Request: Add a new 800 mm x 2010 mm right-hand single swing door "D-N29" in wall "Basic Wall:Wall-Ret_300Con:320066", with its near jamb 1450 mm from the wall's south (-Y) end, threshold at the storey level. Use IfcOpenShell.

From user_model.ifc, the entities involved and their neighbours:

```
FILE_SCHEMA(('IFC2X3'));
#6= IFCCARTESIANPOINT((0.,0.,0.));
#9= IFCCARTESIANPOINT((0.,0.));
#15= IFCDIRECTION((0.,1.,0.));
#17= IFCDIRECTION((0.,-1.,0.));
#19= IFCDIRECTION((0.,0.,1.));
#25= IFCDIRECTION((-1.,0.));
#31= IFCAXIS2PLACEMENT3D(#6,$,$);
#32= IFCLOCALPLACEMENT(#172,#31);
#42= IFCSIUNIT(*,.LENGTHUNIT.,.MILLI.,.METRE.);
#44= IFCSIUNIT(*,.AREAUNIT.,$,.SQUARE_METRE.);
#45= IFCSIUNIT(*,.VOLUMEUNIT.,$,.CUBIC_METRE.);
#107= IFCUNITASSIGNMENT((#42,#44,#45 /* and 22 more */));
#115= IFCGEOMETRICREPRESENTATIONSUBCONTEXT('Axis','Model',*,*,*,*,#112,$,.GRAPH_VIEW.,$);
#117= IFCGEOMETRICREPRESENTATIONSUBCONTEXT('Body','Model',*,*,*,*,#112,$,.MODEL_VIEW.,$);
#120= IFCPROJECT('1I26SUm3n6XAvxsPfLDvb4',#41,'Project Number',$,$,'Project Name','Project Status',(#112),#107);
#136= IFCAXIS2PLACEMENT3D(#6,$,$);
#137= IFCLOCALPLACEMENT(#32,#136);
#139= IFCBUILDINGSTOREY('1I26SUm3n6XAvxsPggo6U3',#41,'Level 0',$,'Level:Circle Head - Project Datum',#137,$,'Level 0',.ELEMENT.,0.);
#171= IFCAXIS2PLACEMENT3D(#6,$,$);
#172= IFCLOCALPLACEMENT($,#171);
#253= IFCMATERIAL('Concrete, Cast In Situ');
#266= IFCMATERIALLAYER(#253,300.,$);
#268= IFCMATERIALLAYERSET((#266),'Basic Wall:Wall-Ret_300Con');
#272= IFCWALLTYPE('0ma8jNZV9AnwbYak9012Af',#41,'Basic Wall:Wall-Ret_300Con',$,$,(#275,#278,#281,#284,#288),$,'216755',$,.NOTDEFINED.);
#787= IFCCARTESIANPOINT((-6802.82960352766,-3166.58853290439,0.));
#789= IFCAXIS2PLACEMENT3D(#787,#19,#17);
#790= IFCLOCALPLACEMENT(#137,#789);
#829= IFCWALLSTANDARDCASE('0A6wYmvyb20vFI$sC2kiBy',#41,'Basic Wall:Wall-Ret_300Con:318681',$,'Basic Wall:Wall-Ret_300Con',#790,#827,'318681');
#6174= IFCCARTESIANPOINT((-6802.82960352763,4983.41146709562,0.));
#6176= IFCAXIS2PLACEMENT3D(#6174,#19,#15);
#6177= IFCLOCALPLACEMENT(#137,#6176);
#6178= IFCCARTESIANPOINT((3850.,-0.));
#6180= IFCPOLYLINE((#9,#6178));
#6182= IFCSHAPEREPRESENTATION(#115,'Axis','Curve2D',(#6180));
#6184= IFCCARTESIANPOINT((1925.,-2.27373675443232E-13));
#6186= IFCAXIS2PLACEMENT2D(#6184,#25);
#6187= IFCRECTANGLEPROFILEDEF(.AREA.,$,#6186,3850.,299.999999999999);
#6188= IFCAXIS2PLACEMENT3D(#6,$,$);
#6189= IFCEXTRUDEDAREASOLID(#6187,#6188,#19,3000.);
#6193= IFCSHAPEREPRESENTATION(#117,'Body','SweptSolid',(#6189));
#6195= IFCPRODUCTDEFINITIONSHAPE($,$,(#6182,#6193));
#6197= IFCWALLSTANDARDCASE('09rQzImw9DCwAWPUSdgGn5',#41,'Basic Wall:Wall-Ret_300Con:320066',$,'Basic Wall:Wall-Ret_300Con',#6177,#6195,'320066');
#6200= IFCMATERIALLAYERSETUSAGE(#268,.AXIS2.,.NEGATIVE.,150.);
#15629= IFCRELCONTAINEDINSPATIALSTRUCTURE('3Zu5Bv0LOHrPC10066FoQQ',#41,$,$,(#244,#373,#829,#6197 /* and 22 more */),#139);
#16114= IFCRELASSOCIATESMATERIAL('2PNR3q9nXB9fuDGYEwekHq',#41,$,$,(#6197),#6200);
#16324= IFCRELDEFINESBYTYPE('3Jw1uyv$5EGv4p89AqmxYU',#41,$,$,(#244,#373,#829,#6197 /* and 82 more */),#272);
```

```python
import numpy as np
import ifcopenshell
import ifcopenshell.api.feature
import ifcopenshell.api.geometry
import ifcopenshell.api.root
import ifcopenshell.api.spatial
import ifcopenshell.api.type
import ifcopenshell.geom
import ifcopenshell.util.element
import ifcopenshell.util.placement
import ifcopenshell.util.representation
import ifcopenshell.util.shape
import ifcopenshell.util.unit

model = ifcopenshell.open("user_model.ifc")
unit_scale = ifcopenshell.util.unit.calculate_unit_scale(model)
settings = ifcopenshell.geom.settings()


def volume(element):
    """Net volume in cubic metres, openings subtracted."""
    shape = ifcopenshell.geom.create_shape(settings, element)
    return ifcopenshell.util.shape.get_volume(shape.geometry)


wall = model.by_id(6197)
storey = ifcopenshell.util.element.get_container(wall, ifc_class="IfcBuildingStorey")
context = ifcopenshell.util.representation.get_context(model, "Model", "Body", "MODEL_VIEW")
before = volume(wall)

width, height, from_end, sill = 0.8, 2.01, 1.45, 0.0  # metres

# The wall runs along its own X axis, and the end named is its -X end.
wall_shape = ifcopenshell.geom.create_shape(settings, wall)
x, y, z = ifcopenshell.util.shape.get_vertices(wall_shape.geometry).T
start = x.min() + from_end
face, thickness = float(y.min()), float(y.max() - y.min())
wall_matrix = ifcopenshell.util.placement.get_local_placement(wall.ObjectPlacement)
level = ifcopenshell.util.placement.get_local_placement(storey.ObjectPlacement)[2, 3]


def in_wall(x, y):
    """Placement at x, y metres in the wall's axes, at sill height."""
    matrix = wall_matrix.copy()
    matrix[:, 3] = wall_matrix @ np.array([x / unit_scale, y / unit_scale, 0.0, 1.0])
    matrix[2, 3] = level + sill / unit_scale
    return matrix


# Opening: a box that overshoots both wall faces by 50 mm.
opening = ifcopenshell.api.root.create_entity(model, ifc_class="IfcOpeningElement")
box = ifcopenshell.api.geometry.add_wall_representation(
    model, context=context, length=width, height=height, thickness=thickness + 0.1
)
ifcopenshell.api.geometry.assign_representation(model, product=opening, representation=box)
ifcopenshell.api.geometry.edit_object_placement(model, product=opening, matrix=in_wall(start, face - 0.05), is_si=False)
ifcopenshell.api.feature.add_feature(model, feature=opening, element=wall)

door = ifcopenshell.api.root.create_entity(model, ifc_class="IfcDoor", name="D-N29")
door.OverallWidth, door.OverallHeight = width / unit_scale, height / unit_scale
body = ifcopenshell.api.geometry.add_door_representation(
    model,
    context=context,
    overall_width=door.OverallWidth,
    overall_height=door.OverallHeight,
    operation_type="SINGLE_SWING_RIGHT",
    lining_properties={"LiningDepth": thickness / unit_scale, "ThresholdDepth": thickness / unit_scale},
)
ifcopenshell.api.geometry.assign_representation(model, product=door, representation=body)
ifcopenshell.api.spatial.assign_container(model, products=[door], relating_structure=storey)
fills = ifcopenshell.api.feature.add_filling(model, opening=opening, element=door)
fills.OwnerHistory = door.OwnerHistory  # required in IFC2X3

# IFC2X3 keeps the operation on the door style.
style = ifcopenshell.api.root.create_entity(model, ifc_class="IfcDoorStyle", name="D-N29")
style.OperationType, style.ConstructionType = "SINGLE_SWING_RIGHT", "NOTDEFINED"
style.ParameterTakesPrecedence = style.Sizeable = False
ifcopenshell.api.type.assign_type(model, related_objects=[door], relating_type=style)

# The lining spans the wall, so the door starts at the wall face.
ifcopenshell.api.geometry.edit_object_placement(model, product=door, matrix=in_wall(start, face), is_si=False)

after = volume(wall)

print(f"wall volume {before:.3f} -> {after:.3f} m3")

model.write("user_model_rev.ifc")
```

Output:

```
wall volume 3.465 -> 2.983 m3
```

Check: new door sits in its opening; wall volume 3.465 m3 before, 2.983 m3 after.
